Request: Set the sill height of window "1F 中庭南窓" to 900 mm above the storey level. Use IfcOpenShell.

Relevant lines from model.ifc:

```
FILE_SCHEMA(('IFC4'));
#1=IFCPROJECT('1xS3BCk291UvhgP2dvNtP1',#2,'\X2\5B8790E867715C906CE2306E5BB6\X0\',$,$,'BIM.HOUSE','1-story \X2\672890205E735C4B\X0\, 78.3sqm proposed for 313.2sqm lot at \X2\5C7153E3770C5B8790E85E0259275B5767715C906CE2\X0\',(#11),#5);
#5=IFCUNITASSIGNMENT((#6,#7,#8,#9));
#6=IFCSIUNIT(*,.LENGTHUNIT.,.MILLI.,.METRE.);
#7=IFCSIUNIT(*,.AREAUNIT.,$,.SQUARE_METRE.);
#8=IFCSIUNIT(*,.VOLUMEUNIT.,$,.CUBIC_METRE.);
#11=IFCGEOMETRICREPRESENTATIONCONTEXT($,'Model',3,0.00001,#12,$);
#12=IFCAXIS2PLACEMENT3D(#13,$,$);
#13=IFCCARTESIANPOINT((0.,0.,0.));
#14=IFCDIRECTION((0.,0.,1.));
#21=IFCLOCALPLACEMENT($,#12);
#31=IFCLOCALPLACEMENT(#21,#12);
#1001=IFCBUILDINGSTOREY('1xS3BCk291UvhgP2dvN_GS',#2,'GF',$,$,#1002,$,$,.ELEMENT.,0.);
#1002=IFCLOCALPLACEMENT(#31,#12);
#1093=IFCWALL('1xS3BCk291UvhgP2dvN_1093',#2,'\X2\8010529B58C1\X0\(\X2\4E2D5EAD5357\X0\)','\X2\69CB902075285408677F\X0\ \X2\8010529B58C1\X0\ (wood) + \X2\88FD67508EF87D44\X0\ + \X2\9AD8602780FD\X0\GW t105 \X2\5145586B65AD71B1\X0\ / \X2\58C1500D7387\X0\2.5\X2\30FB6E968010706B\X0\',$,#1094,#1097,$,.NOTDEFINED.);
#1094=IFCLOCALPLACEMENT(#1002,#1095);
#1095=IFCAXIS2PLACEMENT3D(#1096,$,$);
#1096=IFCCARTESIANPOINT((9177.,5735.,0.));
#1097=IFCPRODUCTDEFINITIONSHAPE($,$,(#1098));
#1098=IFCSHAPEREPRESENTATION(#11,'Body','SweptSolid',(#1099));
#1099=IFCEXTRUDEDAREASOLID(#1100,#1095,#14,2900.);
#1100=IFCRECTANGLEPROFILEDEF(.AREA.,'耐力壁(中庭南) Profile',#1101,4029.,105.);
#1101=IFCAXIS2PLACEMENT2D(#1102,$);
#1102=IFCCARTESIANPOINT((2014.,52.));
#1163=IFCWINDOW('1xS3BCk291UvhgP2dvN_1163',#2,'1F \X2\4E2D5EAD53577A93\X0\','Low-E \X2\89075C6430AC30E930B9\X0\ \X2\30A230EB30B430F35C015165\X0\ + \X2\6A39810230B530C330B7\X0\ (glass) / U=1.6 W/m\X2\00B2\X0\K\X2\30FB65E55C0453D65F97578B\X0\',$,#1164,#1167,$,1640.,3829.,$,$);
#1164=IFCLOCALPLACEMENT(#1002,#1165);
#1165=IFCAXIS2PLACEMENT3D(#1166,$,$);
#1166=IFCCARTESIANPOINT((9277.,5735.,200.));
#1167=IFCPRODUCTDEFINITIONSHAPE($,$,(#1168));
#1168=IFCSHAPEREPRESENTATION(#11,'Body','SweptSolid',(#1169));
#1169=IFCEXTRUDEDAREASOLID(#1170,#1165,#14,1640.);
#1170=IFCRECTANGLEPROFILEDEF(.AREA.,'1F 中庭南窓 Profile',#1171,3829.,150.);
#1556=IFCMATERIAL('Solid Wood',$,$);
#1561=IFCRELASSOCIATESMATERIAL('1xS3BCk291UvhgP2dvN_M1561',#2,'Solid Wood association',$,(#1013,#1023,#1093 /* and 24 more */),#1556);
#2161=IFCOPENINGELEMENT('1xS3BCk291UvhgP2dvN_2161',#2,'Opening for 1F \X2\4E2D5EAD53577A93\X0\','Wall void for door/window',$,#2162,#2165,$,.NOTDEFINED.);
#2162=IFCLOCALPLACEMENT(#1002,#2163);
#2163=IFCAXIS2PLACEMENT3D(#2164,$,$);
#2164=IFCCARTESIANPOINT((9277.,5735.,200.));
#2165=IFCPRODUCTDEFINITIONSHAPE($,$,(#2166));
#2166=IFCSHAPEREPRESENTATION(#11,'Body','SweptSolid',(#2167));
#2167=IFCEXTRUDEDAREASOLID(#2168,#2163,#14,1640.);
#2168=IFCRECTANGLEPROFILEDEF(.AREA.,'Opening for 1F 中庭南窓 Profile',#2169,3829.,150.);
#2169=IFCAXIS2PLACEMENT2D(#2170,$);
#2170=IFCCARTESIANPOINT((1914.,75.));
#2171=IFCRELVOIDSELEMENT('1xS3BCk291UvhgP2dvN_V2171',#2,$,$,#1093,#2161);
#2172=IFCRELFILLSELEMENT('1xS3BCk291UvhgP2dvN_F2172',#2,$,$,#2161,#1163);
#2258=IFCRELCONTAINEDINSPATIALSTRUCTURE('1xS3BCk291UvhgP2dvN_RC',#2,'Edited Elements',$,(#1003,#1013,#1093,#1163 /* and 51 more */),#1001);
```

```python
import numpy as np
import ifcopenshell
import ifcopenshell.api.geometry
import ifcopenshell.geom
import ifcopenshell.util.element
import ifcopenshell.util.placement
import ifcopenshell.util.shape
import ifcopenshell.util.unit

model = ifcopenshell.open("model.ifc")
unit_scale = ifcopenshell.util.unit.calculate_unit_scale(model)

window = model.by_guid("1xS3BCk291UvhgP2dvN_1163")
opening = window.FillsVoids[0].RelatingOpeningElement
storey = ifcopenshell.util.element.get_container(window, ifc_class="IfcBuildingStorey")
level = ifcopenshell.util.placement.get_local_placement(storey.ObjectPlacement)[2, 3]

# The opening's origin need not be at the sill, so measure its lowest point.
shape = ifcopenshell.geom.create_shape(ifcopenshell.geom.settings(), opening)
bottom = ifcopenshell.util.shape.get_shape_bottom_elevation(shape, shape.geometry) / unit_scale
dz = level + 0.9 / unit_scale - bottom

shift = np.array([0.0, 0.0, dz])
# The window is not placed relative to its opening, so move both.
for product in (opening, window):
    matrix = ifcopenshell.util.placement.get_local_placement(product.ObjectPlacement)
    matrix[:3, 3] += shift
    ifcopenshell.api.geometry.edit_object_placement(model, product=product, matrix=matrix, is_si=False)

print(f"moved by {dz * unit_scale:+.3f} m")

model.write("model_v2.ifc")
```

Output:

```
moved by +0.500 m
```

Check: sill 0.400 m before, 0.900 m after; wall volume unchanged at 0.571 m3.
